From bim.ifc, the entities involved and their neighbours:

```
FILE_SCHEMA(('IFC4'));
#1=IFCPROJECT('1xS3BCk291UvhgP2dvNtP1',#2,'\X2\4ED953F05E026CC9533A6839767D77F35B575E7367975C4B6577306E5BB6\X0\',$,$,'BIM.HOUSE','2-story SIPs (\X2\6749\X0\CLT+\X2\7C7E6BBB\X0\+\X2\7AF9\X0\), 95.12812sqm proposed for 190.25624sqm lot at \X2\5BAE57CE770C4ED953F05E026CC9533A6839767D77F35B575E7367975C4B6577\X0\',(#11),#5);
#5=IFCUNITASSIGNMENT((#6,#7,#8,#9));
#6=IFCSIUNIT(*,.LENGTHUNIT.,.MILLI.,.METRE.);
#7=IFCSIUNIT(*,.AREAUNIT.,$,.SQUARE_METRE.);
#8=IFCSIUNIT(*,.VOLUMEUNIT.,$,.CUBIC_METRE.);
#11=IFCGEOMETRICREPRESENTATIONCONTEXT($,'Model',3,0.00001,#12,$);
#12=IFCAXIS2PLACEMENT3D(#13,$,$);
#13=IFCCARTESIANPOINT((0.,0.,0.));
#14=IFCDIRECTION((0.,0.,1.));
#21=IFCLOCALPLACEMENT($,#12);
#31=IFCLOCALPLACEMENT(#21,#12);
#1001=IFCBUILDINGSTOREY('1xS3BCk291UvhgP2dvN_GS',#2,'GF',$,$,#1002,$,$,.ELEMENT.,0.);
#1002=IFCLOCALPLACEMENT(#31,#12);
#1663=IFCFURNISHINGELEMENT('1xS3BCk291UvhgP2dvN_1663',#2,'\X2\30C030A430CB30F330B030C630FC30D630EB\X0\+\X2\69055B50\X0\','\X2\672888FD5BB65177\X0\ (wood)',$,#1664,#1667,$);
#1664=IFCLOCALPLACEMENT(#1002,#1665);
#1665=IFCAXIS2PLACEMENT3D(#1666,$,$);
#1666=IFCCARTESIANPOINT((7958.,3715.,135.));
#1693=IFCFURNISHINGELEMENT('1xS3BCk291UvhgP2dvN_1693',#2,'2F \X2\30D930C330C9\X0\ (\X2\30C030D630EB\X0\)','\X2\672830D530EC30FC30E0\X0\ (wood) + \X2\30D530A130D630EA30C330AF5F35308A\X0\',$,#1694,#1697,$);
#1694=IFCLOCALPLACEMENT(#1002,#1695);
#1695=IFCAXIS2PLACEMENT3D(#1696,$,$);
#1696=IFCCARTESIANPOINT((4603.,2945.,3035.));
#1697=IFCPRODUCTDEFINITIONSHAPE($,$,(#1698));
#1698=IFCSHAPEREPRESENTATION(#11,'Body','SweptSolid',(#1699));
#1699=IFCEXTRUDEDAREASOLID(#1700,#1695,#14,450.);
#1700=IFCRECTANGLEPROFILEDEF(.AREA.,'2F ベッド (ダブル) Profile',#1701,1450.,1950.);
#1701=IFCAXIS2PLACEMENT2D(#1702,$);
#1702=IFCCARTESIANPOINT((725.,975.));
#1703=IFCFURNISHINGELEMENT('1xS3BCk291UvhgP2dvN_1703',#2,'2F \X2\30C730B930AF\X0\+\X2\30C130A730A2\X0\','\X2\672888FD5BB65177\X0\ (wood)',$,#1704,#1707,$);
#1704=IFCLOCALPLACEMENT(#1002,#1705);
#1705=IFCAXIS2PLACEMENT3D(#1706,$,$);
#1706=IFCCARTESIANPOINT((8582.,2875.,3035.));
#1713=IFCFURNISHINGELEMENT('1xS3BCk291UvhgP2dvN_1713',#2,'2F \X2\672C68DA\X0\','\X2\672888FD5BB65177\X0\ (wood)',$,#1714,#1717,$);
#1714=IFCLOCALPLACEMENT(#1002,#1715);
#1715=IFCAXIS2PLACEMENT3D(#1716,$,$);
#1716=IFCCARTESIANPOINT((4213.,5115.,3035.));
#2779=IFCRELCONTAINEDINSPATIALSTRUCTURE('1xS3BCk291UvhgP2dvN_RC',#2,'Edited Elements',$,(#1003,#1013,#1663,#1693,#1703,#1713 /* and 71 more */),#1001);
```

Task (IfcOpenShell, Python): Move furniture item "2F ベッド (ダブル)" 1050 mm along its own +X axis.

```python
import ifcopenshell
import ifcopenshell.api.geometry
import ifcopenshell.util.placement

model = ifcopenshell.open("bim.ifc")

item = model.by_id(1693)
matrix = ifcopenshell.util.placement.get_local_placement(item.ObjectPlacement)
matrix[:3, 3] += matrix[:3, 0] * 1050.0
ifcopenshell.api.geometry.edit_object_placement(model, product=item, matrix=matrix, is_si=False)

print(ifcopenshell.util.placement.get_local_placement(item.ObjectPlacement).round(3) + 0.0)

model.write("bim_updated.ifc")
```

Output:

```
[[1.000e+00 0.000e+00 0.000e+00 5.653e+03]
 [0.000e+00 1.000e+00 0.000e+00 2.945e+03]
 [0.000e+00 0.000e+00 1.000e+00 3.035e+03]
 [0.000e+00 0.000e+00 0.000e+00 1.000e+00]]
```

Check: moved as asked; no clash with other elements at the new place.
